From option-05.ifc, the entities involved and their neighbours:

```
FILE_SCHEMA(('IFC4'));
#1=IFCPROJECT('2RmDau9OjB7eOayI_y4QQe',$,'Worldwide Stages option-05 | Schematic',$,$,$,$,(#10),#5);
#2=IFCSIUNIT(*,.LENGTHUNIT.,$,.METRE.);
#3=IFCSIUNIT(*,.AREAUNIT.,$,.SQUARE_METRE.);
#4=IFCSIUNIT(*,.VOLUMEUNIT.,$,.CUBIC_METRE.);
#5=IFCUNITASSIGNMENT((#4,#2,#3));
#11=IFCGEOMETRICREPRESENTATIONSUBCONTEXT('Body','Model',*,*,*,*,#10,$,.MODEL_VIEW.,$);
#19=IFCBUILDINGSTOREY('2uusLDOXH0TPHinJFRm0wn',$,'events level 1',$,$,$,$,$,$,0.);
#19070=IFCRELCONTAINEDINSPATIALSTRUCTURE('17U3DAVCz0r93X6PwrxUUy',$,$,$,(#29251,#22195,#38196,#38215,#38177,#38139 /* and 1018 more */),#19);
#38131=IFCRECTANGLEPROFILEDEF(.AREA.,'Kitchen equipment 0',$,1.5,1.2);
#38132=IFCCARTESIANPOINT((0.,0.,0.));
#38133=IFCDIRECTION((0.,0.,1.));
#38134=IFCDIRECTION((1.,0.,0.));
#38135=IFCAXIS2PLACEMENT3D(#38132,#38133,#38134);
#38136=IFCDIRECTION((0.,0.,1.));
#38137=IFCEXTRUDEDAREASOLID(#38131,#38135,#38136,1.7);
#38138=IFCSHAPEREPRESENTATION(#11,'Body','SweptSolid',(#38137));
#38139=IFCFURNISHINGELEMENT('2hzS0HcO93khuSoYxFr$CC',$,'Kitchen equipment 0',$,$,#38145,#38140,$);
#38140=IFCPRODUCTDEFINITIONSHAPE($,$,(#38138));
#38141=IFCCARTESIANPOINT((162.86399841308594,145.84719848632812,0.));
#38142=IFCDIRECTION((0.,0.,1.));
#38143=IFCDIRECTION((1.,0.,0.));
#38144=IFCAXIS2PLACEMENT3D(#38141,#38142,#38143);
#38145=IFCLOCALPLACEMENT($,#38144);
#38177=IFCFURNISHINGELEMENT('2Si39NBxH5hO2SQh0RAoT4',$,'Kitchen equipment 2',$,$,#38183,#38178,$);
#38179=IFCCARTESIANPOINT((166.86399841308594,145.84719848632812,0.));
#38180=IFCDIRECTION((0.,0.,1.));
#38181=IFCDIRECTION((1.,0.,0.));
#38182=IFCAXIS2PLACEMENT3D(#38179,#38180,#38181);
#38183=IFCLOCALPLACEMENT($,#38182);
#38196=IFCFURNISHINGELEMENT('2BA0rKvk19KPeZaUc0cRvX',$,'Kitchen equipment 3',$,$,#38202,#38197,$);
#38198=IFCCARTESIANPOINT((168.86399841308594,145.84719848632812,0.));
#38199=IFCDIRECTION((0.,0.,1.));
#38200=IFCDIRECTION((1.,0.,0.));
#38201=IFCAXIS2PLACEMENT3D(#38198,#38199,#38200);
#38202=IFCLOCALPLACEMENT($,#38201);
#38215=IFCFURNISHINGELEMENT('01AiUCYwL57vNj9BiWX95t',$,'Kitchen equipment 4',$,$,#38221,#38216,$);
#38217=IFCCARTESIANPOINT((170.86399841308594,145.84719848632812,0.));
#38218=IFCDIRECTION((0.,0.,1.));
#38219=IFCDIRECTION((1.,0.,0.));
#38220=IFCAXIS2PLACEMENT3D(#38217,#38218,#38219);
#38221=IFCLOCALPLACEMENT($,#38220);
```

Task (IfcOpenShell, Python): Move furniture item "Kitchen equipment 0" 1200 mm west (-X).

```python
import ifcopenshell
import ifcopenshell.api.geometry
import ifcopenshell.util.placement

model = ifcopenshell.open("option-05.ifc")

item = model.by_guid("2hzS0HcO93khuSoYxFr$CC")
matrix = ifcopenshell.util.placement.get_local_placement(item.ObjectPlacement)
matrix[0, 3] -= 1.2
ifcopenshell.api.geometry.edit_object_placement(model, product=item, matrix=matrix, is_si=False)

print(ifcopenshell.util.placement.get_local_placement(item.ObjectPlacement).round(3) + 0.0)

model.write("option-05_edited.ifc")
```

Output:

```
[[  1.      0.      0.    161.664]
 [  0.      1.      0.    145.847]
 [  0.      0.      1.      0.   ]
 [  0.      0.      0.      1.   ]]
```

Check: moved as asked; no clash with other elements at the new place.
